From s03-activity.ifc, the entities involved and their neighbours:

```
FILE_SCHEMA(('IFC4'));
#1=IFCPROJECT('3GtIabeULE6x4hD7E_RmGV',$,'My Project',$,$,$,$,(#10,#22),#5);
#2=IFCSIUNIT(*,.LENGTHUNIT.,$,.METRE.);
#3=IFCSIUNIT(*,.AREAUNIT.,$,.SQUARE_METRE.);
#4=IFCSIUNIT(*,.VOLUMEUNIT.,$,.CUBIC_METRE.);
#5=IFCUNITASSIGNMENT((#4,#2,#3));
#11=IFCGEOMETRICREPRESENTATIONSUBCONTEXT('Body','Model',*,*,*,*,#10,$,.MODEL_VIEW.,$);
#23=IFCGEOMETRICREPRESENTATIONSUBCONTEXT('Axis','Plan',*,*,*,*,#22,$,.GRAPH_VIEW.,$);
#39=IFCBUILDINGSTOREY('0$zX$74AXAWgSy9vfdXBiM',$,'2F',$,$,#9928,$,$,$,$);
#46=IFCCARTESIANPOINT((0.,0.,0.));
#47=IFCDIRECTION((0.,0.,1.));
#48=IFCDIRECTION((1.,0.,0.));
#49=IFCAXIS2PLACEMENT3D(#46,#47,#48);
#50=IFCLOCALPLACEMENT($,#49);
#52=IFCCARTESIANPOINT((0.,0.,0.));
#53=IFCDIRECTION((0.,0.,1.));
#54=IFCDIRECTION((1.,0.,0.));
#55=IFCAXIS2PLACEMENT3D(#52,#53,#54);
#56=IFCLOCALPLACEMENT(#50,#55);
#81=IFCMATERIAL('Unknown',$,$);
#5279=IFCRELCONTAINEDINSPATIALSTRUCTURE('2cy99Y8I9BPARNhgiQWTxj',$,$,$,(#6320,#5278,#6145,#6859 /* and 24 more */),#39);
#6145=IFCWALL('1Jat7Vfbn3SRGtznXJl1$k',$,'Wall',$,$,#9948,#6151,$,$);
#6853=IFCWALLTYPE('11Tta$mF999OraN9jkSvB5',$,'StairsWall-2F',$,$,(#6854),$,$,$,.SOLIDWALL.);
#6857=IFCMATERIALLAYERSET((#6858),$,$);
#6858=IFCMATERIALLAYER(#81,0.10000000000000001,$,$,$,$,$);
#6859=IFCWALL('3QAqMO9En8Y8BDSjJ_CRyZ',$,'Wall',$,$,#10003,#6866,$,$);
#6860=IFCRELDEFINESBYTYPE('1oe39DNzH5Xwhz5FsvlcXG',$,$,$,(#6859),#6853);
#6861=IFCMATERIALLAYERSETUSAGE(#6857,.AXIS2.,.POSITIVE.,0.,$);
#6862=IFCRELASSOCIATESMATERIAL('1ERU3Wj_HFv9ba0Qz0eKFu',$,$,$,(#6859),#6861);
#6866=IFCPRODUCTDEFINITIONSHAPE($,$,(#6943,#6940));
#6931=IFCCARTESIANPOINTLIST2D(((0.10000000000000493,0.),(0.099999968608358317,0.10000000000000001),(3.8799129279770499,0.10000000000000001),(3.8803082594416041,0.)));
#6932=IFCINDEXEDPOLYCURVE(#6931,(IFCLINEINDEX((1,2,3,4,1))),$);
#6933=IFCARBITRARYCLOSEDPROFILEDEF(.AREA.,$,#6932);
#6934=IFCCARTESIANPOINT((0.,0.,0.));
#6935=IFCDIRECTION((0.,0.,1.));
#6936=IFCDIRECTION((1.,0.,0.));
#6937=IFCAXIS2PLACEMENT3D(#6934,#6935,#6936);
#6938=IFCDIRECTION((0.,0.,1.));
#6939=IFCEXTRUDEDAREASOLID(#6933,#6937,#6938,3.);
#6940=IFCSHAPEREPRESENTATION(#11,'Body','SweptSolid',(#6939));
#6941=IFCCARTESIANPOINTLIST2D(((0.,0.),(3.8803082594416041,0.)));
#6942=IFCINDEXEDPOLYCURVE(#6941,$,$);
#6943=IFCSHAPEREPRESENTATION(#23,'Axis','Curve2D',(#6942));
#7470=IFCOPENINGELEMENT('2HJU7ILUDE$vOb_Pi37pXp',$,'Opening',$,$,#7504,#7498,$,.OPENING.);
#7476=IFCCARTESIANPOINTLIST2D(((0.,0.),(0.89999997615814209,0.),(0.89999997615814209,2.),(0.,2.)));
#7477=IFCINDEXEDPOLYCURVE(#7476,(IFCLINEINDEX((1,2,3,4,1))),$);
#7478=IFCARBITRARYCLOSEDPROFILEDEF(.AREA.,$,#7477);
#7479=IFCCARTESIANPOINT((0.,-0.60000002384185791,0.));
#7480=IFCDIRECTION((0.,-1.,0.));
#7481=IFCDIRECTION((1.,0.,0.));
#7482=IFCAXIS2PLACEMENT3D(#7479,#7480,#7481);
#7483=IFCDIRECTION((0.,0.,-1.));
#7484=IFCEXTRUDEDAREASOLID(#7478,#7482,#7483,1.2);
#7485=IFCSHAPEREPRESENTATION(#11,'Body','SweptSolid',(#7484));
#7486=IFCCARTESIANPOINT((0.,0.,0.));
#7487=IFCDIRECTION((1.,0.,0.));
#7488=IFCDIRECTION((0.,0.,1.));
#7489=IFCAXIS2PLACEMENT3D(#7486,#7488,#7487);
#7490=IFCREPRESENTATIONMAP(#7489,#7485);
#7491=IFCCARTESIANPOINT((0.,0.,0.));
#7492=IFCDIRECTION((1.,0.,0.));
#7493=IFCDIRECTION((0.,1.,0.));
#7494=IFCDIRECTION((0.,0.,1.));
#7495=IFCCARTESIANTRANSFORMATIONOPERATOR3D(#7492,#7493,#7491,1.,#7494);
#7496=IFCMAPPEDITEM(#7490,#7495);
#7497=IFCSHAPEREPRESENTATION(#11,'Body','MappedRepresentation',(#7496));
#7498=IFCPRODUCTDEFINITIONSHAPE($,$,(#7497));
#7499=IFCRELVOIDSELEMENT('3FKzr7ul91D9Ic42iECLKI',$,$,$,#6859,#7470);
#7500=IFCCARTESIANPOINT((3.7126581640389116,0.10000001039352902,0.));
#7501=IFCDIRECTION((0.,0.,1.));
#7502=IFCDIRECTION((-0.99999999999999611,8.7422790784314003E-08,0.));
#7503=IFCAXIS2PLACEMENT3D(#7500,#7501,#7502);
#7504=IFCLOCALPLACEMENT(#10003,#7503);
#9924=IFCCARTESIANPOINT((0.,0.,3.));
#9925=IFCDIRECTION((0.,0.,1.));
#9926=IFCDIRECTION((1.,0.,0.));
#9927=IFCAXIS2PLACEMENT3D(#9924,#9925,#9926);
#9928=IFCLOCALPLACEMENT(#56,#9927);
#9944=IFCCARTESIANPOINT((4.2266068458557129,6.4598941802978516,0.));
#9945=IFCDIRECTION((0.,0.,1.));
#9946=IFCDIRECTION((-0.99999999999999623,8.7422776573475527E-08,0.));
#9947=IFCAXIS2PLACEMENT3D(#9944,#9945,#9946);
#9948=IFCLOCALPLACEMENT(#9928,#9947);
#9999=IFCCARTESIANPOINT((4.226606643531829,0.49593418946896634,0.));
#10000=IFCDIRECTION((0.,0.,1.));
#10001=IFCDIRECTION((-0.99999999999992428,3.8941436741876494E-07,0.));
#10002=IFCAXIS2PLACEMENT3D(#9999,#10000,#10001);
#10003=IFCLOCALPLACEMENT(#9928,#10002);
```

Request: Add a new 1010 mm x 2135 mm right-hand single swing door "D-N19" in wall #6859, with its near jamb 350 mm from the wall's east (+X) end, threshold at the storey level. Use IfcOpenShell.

```python
import numpy as np
import ifcopenshell
import ifcopenshell.api.feature
import ifcopenshell.api.geometry
import ifcopenshell.api.root
import ifcopenshell.api.spatial
import ifcopenshell.geom
import ifcopenshell.util.element
import ifcopenshell.util.placement
import ifcopenshell.util.representation
import ifcopenshell.util.shape
import ifcopenshell.util.unit

model = ifcopenshell.open("s03-activity.ifc")
unit_scale = ifcopenshell.util.unit.calculate_unit_scale(model)
settings = ifcopenshell.geom.settings()


def volume(element):
    """Net volume in cubic metres, openings subtracted."""
    shape = ifcopenshell.geom.create_shape(settings, element)
    return ifcopenshell.util.shape.get_volume(shape.geometry)


wall = model.by_guid("3QAqMO9En8Y8BDSjJ_CRyZ")
storey = ifcopenshell.util.element.get_container(wall, ifc_class="IfcBuildingStorey")
context = ifcopenshell.util.representation.get_context(model, "Model", "Body", "MODEL_VIEW")
before = volume(wall)

width, height, from_end, sill = 1.01, 2.135, 0.35, 0.0  # metres

# The wall runs along its own X axis, and the end named is its -X end.
wall_shape = ifcopenshell.geom.create_shape(settings, wall)
x, y, z = ifcopenshell.util.shape.get_vertices(wall_shape.geometry).T
start = x.min() + from_end
face, thickness = float(y.min()), float(y.max() - y.min())
wall_matrix = ifcopenshell.util.placement.get_local_placement(wall.ObjectPlacement)
level = ifcopenshell.util.placement.get_local_placement(storey.ObjectPlacement)[2, 3]


def in_wall(x, y):
    """Placement at x, y metres in the wall's axes, at sill height."""
    matrix = wall_matrix.copy()
    matrix[:, 3] = wall_matrix @ np.array([x / unit_scale, y / unit_scale, 0.0, 1.0])
    matrix[2, 3] = level + sill / unit_scale
    return matrix


# Opening: a box that overshoots both wall faces by 50 mm.
opening = ifcopenshell.api.root.create_entity(model, ifc_class="IfcOpeningElement", predefined_type="OPENING")
box = ifcopenshell.api.geometry.add_wall_representation(
    model, context=context, length=width, height=height, thickness=thickness + 0.1
)
ifcopenshell.api.geometry.assign_representation(model, product=opening, representation=box)
ifcopenshell.api.geometry.edit_object_placement(model, product=opening, matrix=in_wall(start, face - 0.05), is_si=False)
ifcopenshell.api.feature.add_feature(model, feature=opening, element=wall)

door = ifcopenshell.api.root.create_entity(model, ifc_class="IfcDoor", name="D-N19", predefined_type="DOOR")
door.OverallWidth, door.OverallHeight = width / unit_scale, height / unit_scale
door.OperationType = "SINGLE_SWING_RIGHT"
body = ifcopenshell.api.geometry.add_door_representation(
    model,
    context=context,
    overall_width=door.OverallWidth,
    overall_height=door.OverallHeight,
    operation_type="SINGLE_SWING_RIGHT",
    lining_properties={"LiningDepth": thickness / unit_scale, "ThresholdDepth": thickness / unit_scale},
)
ifcopenshell.api.geometry.assign_representation(model, product=door, representation=body)
ifcopenshell.api.spatial.assign_container(model, products=[door], relating_structure=storey)
ifcopenshell.api.feature.add_filling(model, opening=opening, element=door)

# The lining spans the wall, so the door starts at the wall face.
ifcopenshell.api.geometry.edit_object_placement(model, product=door, matrix=in_wall(start, face), is_si=False)

after = volume(wall)

print(f"wall volume {before:.3f} -> {after:.3f} m3")

model.write("s03-activity-out.ifc")
```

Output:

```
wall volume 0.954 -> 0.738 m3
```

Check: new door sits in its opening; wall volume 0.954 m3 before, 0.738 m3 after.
